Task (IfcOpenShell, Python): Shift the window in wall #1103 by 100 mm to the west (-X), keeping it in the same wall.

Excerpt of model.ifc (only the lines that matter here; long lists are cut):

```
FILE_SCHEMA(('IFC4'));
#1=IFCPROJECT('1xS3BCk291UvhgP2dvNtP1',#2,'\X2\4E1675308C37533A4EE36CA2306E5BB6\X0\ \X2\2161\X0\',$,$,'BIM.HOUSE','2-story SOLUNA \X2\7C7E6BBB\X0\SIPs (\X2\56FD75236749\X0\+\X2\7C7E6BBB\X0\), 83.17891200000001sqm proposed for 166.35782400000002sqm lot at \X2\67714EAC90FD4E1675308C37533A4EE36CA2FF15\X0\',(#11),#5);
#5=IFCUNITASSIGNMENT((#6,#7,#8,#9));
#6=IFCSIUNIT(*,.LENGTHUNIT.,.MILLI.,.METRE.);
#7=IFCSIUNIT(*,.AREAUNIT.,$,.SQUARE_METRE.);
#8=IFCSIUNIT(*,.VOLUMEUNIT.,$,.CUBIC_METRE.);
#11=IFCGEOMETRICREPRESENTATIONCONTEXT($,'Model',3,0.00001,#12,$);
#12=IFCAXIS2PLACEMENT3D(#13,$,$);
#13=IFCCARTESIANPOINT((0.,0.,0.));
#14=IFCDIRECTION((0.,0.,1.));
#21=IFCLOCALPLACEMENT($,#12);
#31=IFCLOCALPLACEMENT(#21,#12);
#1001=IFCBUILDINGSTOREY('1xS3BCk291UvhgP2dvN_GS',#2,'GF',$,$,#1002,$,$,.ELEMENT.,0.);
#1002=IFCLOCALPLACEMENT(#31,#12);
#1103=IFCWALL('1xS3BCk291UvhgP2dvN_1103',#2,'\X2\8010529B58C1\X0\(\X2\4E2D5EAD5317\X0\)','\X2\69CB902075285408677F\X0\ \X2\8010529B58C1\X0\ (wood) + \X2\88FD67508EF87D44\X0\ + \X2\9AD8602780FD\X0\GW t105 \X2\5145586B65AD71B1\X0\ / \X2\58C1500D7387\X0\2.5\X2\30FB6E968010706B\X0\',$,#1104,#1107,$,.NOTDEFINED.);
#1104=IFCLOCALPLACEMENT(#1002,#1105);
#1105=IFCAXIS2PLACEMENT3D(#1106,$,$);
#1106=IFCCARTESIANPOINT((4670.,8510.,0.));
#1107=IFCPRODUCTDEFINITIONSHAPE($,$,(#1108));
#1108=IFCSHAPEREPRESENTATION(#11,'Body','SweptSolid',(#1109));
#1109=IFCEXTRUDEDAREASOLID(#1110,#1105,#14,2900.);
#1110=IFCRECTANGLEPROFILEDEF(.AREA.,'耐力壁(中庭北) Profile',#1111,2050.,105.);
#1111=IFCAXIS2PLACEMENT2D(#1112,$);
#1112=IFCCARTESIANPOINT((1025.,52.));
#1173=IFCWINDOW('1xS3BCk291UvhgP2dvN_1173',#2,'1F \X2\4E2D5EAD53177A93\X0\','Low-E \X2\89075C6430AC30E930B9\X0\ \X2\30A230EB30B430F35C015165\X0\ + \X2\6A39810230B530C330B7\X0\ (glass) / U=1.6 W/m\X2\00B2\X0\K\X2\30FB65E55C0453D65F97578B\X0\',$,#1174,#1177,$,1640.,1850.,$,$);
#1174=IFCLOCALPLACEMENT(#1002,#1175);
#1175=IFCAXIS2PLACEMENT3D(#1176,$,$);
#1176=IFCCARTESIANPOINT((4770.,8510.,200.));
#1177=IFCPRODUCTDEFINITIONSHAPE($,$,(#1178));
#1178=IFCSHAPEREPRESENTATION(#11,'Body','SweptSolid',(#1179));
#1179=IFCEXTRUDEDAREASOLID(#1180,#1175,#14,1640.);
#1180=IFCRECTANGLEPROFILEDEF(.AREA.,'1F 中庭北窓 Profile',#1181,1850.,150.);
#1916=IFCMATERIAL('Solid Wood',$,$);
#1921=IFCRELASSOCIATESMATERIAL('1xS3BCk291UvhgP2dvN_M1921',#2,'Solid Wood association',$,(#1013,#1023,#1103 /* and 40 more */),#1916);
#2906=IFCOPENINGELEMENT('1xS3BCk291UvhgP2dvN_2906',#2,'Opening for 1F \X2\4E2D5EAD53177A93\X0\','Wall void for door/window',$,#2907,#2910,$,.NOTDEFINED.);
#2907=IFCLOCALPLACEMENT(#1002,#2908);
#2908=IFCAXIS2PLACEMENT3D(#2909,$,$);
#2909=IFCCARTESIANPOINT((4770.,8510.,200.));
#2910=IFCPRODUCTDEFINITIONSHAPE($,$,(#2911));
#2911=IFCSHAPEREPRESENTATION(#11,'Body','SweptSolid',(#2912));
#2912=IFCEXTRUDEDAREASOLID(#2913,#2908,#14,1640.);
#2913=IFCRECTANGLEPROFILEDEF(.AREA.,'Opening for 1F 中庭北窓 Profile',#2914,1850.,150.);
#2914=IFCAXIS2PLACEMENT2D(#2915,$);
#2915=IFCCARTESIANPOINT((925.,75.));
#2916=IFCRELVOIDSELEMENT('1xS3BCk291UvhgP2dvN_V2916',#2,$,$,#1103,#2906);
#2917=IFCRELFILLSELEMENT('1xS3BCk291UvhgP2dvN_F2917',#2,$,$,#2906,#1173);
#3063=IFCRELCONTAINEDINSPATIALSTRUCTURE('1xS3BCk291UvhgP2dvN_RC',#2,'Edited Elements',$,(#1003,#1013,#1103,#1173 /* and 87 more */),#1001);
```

```python
import ifcopenshell
import ifcopenshell.api.geometry
import ifcopenshell.util.placement

model = ifcopenshell.open("model.ifc")

window = model.by_guid("1xS3BCk291UvhgP2dvN_1173")
opening = window.FillsVoids[0].RelatingOpeningElement
wall = opening.VoidsElements[0].RelatingBuildingElement

wall_matrix = ifcopenshell.util.placement.get_local_placement(wall.ObjectPlacement)
shift = wall_matrix[:3, 0] * -100.0
before = ifcopenshell.util.placement.get_local_placement(window.ObjectPlacement)[:3, 3].copy()

# The window is not placed relative to its opening, so move both.
for product in (opening, window):
    matrix = ifcopenshell.util.placement.get_local_placement(product.ObjectPlacement)
    matrix[:3, 3] += shift
    ifcopenshell.api.geometry.edit_object_placement(model, product=product, matrix=matrix, is_si=False)

after = ifcopenshell.util.placement.get_local_placement(window.ObjectPlacement)[:3, 3]
print("window moved by", (after - before).round(3) + 0.0)

model.write("model_rev.ifc")
```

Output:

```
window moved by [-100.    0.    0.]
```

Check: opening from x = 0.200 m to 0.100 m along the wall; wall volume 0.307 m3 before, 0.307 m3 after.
